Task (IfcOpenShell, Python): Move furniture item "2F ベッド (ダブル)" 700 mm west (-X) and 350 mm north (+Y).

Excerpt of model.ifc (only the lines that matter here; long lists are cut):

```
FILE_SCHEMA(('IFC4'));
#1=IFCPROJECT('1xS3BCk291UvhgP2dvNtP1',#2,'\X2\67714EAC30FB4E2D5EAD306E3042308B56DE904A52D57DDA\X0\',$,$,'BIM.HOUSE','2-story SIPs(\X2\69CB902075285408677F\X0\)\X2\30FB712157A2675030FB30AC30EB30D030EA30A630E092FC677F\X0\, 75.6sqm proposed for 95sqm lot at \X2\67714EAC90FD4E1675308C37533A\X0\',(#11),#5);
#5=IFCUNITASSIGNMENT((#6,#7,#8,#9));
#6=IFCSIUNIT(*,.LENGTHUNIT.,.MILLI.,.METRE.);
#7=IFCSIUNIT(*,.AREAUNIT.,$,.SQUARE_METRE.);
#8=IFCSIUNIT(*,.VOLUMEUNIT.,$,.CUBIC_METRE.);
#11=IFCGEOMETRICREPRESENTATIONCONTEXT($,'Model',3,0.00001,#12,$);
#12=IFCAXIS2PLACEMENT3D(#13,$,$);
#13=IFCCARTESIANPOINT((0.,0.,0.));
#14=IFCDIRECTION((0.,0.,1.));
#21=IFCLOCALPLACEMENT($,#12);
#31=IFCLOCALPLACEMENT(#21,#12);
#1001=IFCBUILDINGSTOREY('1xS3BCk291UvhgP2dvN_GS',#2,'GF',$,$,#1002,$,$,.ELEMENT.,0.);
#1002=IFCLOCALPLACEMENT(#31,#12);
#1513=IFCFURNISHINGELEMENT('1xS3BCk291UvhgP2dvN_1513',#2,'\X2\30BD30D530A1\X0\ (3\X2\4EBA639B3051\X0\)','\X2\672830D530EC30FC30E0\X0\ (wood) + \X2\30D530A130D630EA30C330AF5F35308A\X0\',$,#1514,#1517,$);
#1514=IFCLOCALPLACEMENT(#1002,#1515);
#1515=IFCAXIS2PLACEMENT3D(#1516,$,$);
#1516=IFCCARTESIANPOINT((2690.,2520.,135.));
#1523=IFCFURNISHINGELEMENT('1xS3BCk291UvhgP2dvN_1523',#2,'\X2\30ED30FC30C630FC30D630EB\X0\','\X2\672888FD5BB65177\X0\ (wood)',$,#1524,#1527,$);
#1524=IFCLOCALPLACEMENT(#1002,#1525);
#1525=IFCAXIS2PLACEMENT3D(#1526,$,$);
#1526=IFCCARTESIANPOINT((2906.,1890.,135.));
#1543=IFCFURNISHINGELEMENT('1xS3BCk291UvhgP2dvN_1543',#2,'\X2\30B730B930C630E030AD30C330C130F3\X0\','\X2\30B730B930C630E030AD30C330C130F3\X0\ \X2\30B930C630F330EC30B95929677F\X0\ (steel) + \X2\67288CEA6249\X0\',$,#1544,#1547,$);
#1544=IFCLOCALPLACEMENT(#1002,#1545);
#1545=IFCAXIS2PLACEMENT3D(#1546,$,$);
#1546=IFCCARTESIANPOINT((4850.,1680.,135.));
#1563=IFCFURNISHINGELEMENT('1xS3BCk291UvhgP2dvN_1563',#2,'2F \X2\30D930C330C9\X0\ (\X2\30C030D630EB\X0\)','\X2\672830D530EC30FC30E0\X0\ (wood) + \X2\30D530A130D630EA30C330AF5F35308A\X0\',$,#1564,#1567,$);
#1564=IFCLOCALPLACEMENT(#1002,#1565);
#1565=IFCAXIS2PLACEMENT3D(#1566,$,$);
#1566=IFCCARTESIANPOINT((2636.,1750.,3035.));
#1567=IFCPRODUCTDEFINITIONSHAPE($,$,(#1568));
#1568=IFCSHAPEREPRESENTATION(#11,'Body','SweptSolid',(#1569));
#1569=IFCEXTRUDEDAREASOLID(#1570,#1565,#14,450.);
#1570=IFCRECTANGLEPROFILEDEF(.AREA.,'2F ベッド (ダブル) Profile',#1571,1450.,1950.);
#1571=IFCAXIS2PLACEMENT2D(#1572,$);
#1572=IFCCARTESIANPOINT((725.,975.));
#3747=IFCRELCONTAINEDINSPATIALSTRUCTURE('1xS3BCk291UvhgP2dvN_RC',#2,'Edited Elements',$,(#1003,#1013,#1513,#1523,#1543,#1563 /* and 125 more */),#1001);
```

```python
import ifcopenshell
import ifcopenshell.api.geometry
import ifcopenshell.util.placement
import ifcopenshell.util.unit

model = ifcopenshell.open("model.ifc")
unit_scale = ifcopenshell.util.unit.calculate_unit_scale(model)

item = model.by_guid("1xS3BCk291UvhgP2dvN_1563")
matrix = ifcopenshell.util.placement.get_local_placement(item.ObjectPlacement)
matrix[0, 3] -= 0.7 / unit_scale
matrix[1, 3] += 0.35 / unit_scale
ifcopenshell.api.geometry.edit_object_placement(model, product=item, matrix=matrix, is_si=False)

print(ifcopenshell.util.placement.get_local_placement(item.ObjectPlacement).round(3) + 0.0)

model.write("model-out.ifc")
```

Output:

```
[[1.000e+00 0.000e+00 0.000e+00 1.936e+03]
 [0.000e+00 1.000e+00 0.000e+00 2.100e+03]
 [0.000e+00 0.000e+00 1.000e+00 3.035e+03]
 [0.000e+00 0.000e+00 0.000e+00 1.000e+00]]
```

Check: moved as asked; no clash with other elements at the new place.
